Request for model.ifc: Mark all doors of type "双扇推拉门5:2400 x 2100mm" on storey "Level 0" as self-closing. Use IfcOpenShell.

First a look at what the model holds.

```python
import ifcopenshell
import ifcopenshell.util.element

model = ifcopenshell.open("model.ifc")
print(model.schema)
storey = next(s for s in model.by_type("IfcBuildingStorey") if s.Name == "Level 0")
doors = [e for e in ifcopenshell.util.element.get_decomposition(storey) if e.is_a("IfcDoor")]
seen = {}
for e in doors:
    element_type = ifcopenshell.util.element.get_type(e)
    key = (element_type.Name if element_type != e and element_type else None, ifcopenshell.util.element.get_pset(e, "Pset_DoorCommon", "SelfClosing"))
    seen[key] = seen.get(key, 0) + 1
for (name, value), count in sorted(seen.items(), key=str):
    print(count, "x", name, "|", value)
```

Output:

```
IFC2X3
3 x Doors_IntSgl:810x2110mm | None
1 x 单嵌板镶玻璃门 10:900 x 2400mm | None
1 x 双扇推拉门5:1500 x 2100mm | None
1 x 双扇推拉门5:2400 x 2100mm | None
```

```python
import ifcopenshell
import ifcopenshell.api.pset
import ifcopenshell.util.element

model = ifcopenshell.open("model.ifc")

storey = next(s for s in model.by_type("IfcBuildingStorey") if s.Name == "Level 0")
doors = [e for e in ifcopenshell.util.element.get_decomposition(storey) if e.is_a("IfcDoor")]

count = 0
for e in doors:
    element_type = ifcopenshell.util.element.get_type(e)
    if element_type in (None, e) or element_type.Name != "双扇推拉门5:2400 x 2100mm":
        continue
    # add_pset returns the element's existing set when there is one.
    pset = ifcopenshell.api.pset.add_pset(model, product=e, name="Pset_DoorCommon")
    ifcopenshell.api.pset.edit_pset(model, pset=pset, properties={"SelfClosing": True})
    count += 1

print(count, "doors updated")

model.write("model-out.ifc")
```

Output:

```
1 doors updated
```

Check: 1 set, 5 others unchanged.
